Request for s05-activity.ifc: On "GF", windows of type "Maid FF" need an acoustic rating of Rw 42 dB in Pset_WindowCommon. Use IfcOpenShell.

First a look at what the model holds.

```python
import ifcopenshell
import ifcopenshell.util.element

model = ifcopenshell.open("s05-activity.ifc")
print(model.schema)
storey = next(s for s in model.by_type("IfcBuildingStorey") if s.Name == "GF")
windows = [e for e in ifcopenshell.util.element.get_decomposition(storey) if e.is_a("IfcWindow")]
seen = {}
for e in windows:
    element_type = ifcopenshell.util.element.get_type(e)
    key = (element_type.Name if element_type != e and element_type else None, ifcopenshell.util.element.get_pset(e, "Pset_WindowCommon", "AcousticRating"))
    seen[key] = seen.get(key, 0) + 1
for (name, value), count in sorted(seen.items(), key=str):
    print(count, "x", name, "|", value)
```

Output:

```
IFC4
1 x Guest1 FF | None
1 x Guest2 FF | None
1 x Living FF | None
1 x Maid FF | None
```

```python
import ifcopenshell
import ifcopenshell.api.pset
import ifcopenshell.util.element

model = ifcopenshell.open("s05-activity.ifc")

storey = next(s for s in model.by_type("IfcBuildingStorey") if s.Name == "GF")
windows = [e for e in ifcopenshell.util.element.get_decomposition(storey) if e.is_a("IfcWindow")]

count = 0
for e in windows:
    element_type = ifcopenshell.util.element.get_type(e)
    if element_type in (None, e) or element_type.Name != "Maid FF":
        continue
    # add_pset returns the element's existing set when there is one.
    pset = ifcopenshell.api.pset.add_pset(model, product=e, name="Pset_WindowCommon")
    ifcopenshell.api.pset.edit_pset(model, pset=pset, properties={"AcousticRating": "Rw 42 dB"})
    count += 1

print(count, "windows updated")

model.write("s05-activity-out.ifc")
```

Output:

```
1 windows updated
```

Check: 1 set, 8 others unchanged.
